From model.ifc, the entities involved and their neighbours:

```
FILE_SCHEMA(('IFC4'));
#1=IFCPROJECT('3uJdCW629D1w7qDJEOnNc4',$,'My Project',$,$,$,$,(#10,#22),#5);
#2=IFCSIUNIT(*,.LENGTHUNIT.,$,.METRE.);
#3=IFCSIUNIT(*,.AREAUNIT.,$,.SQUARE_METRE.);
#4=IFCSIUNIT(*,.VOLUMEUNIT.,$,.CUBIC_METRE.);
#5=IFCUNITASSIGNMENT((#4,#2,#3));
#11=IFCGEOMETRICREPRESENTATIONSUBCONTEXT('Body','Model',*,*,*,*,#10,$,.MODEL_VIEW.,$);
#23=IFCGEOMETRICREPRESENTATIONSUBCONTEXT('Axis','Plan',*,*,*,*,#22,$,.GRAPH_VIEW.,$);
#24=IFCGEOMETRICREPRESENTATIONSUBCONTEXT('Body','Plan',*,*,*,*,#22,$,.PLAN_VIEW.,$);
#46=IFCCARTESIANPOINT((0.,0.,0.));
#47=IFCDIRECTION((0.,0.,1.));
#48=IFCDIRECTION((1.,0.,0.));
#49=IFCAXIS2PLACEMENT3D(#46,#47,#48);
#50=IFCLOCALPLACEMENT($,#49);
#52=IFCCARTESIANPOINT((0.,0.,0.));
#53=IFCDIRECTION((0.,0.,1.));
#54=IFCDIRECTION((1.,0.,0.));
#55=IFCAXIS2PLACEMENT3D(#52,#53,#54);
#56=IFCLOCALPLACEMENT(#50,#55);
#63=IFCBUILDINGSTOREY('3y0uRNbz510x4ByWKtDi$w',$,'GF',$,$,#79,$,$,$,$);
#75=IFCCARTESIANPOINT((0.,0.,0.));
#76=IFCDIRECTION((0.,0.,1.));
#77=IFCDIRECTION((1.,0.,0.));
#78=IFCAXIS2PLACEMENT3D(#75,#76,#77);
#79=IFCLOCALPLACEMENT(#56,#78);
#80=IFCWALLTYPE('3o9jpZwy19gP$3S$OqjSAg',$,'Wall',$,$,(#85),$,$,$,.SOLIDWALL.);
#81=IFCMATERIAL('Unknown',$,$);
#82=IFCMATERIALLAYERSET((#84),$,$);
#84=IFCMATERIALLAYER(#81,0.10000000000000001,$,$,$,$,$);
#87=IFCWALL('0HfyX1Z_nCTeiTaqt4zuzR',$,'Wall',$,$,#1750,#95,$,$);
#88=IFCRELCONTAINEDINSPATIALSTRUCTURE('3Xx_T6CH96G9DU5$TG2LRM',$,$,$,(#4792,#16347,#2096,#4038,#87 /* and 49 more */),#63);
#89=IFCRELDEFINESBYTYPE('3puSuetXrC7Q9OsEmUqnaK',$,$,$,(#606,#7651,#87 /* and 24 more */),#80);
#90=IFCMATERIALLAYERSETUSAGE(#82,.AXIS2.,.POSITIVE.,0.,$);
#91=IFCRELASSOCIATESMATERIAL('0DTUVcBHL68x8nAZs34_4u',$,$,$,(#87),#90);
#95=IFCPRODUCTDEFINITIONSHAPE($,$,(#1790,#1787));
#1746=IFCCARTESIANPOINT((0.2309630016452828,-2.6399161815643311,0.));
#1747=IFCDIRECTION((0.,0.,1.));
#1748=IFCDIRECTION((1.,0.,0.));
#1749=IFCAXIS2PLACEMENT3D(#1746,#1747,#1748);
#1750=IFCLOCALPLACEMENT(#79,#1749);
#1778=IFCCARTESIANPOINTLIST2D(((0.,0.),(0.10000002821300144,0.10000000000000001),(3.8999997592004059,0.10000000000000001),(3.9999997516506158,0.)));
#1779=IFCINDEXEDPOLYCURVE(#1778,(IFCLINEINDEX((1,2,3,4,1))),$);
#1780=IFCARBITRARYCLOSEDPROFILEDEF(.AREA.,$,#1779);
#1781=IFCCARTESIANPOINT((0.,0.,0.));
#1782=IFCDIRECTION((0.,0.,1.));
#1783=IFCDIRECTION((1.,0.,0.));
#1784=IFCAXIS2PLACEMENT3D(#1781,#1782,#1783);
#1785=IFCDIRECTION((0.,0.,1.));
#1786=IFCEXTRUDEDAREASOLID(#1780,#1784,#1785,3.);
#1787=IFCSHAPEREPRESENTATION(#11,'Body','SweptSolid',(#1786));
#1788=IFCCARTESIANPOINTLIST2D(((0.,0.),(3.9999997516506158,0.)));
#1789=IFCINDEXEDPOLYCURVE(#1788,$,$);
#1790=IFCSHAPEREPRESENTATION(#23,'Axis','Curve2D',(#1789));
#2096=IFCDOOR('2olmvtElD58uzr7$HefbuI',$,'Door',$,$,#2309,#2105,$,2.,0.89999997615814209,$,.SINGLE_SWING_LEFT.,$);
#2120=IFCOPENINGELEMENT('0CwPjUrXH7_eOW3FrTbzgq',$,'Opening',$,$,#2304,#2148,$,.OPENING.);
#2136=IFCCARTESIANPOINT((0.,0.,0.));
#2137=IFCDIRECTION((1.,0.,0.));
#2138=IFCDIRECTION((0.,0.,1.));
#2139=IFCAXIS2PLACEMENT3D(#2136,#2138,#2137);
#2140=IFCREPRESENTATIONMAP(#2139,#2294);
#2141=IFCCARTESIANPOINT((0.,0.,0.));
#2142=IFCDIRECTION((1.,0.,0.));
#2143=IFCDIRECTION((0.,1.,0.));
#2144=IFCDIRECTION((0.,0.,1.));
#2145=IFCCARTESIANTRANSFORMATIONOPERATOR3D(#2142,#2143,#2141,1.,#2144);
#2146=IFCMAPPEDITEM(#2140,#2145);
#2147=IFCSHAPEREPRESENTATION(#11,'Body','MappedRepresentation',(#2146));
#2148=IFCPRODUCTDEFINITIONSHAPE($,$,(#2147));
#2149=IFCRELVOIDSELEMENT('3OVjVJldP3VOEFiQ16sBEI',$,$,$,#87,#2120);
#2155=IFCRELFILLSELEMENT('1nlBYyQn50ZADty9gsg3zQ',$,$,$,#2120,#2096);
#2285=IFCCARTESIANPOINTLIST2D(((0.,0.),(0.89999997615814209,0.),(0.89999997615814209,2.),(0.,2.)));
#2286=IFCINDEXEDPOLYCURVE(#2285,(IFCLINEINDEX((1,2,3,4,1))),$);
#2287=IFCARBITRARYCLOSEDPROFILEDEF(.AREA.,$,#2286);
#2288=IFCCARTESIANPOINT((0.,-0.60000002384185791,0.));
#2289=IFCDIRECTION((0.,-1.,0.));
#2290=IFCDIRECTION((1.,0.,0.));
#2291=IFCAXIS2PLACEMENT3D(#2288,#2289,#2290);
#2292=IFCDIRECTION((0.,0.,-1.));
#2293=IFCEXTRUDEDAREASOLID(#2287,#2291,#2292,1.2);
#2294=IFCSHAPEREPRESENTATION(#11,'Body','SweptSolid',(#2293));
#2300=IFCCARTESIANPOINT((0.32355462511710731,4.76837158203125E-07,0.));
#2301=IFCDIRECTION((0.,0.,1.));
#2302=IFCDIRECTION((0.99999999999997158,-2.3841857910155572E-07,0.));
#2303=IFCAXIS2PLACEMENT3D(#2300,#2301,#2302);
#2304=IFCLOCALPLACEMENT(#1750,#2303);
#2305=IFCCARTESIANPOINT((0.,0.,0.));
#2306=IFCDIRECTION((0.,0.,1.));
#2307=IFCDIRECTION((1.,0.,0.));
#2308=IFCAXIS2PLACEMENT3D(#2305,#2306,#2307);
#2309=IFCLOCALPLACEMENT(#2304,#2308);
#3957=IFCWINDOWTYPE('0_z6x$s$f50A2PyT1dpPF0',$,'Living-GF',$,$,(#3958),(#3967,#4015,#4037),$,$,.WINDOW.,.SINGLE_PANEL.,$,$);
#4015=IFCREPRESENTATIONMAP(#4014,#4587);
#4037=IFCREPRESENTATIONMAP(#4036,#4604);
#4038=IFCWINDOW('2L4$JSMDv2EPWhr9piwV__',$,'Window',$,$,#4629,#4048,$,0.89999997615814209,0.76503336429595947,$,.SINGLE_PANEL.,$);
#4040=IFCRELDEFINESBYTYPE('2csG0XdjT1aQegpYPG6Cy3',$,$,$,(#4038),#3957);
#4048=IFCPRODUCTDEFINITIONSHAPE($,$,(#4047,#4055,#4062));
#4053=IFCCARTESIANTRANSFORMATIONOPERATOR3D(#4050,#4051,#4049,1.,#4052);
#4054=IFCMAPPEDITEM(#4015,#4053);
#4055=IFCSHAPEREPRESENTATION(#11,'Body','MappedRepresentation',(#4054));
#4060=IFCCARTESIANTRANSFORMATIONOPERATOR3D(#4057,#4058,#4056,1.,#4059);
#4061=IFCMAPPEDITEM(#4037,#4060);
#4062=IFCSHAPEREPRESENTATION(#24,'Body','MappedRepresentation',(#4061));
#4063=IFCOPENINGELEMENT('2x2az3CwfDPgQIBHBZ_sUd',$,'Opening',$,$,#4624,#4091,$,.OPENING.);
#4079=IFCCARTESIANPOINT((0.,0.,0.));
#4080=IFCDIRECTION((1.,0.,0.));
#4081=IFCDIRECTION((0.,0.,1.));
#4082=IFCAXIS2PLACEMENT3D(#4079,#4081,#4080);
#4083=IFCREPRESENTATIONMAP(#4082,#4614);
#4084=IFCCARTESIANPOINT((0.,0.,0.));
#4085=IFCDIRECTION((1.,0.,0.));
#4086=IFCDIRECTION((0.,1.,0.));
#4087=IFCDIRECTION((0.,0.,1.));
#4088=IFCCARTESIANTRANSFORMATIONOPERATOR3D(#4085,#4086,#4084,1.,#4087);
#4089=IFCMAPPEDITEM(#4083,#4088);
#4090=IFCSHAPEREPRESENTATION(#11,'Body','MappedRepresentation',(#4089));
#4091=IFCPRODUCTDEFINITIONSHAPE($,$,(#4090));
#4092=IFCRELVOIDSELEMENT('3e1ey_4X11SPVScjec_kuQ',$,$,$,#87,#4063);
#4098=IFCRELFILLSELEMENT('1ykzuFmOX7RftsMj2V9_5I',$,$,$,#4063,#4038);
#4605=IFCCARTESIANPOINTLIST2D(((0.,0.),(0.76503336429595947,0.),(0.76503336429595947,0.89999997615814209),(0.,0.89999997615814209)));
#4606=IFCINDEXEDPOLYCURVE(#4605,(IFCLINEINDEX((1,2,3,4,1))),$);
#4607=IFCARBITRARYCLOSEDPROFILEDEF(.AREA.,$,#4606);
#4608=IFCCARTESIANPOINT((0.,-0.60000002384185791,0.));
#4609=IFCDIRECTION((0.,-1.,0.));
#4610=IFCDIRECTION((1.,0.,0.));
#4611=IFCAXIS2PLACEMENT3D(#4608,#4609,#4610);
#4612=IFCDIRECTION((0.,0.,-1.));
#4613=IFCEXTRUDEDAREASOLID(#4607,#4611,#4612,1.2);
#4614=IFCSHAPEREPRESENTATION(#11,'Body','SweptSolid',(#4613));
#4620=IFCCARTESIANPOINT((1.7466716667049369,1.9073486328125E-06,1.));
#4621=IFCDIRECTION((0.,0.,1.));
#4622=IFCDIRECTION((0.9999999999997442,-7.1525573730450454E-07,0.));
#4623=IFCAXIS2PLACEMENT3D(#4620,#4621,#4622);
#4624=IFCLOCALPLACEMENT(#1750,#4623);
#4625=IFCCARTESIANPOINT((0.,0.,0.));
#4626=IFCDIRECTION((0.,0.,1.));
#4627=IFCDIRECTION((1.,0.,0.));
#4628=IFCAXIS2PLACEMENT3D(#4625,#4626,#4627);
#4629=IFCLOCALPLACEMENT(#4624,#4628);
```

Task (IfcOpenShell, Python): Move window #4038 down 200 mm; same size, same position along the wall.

```python
import numpy as np
import ifcopenshell
import ifcopenshell.api.geometry
import ifcopenshell.util.placement
import ifcopenshell.util.unit

model = ifcopenshell.open("model.ifc")
unit_scale = ifcopenshell.util.unit.calculate_unit_scale(model)

window = model.by_guid("2L4$JSMDv2EPWhr9piwV__")
opening = window.FillsVoids[0].RelatingOpeningElement
dz = -0.2 / unit_scale

shift = np.array([0.0, 0.0, dz])
# The window is placed relative to its opening, so it follows when the opening moves.
matrix = ifcopenshell.util.placement.get_local_placement(opening.ObjectPlacement)
matrix[:3, 3] += shift
ifcopenshell.api.geometry.edit_object_placement(
    model, product=opening, matrix=matrix, is_si=False, should_transform_children=True
)

print(f"moved by {dz * unit_scale:+.3f} m")

model.write("model_rev.ifc")
```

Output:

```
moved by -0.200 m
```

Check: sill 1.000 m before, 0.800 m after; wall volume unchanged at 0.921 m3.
